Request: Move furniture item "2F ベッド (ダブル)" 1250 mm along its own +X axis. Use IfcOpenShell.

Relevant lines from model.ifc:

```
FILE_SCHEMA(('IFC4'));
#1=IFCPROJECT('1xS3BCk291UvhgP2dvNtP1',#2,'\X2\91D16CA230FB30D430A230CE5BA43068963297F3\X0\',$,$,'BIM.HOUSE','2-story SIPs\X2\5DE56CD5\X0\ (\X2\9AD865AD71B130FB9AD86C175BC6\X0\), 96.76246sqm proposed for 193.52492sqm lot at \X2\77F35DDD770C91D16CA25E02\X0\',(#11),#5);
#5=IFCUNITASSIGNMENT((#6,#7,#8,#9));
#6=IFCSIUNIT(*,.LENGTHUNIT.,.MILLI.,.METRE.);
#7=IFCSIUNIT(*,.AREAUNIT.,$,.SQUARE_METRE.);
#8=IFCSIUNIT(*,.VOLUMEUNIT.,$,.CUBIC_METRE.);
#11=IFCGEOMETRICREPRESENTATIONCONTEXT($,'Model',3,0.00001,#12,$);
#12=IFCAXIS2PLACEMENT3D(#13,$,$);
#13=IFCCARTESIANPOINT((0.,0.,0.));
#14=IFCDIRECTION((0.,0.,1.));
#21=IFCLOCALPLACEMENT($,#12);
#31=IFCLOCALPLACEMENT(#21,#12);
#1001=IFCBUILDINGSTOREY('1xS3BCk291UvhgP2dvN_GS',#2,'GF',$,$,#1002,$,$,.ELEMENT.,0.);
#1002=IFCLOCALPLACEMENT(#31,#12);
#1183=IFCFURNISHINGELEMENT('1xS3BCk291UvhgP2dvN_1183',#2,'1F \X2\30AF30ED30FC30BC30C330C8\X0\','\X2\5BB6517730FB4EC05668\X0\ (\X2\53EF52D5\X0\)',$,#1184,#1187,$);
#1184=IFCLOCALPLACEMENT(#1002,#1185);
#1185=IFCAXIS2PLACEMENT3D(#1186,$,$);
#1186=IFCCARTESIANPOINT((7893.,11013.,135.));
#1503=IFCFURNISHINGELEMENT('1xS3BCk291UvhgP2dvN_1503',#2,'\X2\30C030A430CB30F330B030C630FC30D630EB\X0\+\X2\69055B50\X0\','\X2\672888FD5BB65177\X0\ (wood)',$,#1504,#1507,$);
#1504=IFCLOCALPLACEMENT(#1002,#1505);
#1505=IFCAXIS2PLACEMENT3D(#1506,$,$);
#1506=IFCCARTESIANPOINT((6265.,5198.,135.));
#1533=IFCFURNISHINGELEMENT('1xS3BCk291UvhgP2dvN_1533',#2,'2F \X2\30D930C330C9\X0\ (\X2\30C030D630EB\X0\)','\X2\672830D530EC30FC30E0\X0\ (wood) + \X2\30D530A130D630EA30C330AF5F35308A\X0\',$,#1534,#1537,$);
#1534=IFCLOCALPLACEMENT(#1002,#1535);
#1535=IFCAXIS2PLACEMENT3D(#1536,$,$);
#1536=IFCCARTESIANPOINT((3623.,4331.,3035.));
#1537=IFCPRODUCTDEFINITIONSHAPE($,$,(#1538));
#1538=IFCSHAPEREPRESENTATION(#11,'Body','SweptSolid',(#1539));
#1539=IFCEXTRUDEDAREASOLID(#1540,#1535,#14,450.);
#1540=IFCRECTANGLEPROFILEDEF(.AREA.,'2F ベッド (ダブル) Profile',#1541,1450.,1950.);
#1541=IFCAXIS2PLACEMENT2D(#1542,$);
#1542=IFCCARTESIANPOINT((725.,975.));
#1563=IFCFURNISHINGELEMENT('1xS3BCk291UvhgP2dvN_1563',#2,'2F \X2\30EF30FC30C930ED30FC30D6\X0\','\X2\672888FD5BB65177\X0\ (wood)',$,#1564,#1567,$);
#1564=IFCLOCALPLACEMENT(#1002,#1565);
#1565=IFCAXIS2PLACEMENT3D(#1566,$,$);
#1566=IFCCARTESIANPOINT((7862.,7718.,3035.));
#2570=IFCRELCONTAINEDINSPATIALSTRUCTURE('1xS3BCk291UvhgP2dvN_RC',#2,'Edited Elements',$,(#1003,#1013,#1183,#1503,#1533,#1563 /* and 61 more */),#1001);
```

```python
import ifcopenshell
import ifcopenshell.api.geometry
import ifcopenshell.util.placement
import ifcopenshell.util.unit

model = ifcopenshell.open("model.ifc")
unit_scale = ifcopenshell.util.unit.calculate_unit_scale(model)

item = model.by_id(1533)
matrix = ifcopenshell.util.placement.get_local_placement(item.ObjectPlacement)
matrix[:3, 3] += matrix[:3, 0] * 1.25 / unit_scale
ifcopenshell.api.geometry.edit_object_placement(model, product=item, matrix=matrix, is_si=False)

print(ifcopenshell.util.placement.get_local_placement(item.ObjectPlacement).round(3) + 0.0)

model.write("model_edited.ifc")
```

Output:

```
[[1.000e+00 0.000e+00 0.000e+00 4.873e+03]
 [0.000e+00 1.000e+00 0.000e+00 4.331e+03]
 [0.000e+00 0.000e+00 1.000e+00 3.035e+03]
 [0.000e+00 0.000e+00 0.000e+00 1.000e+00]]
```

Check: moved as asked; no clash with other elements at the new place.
